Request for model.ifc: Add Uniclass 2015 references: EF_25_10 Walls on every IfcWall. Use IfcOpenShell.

First a look at what the model holds.

```python
import ifcopenshell

model = ifcopenshell.open("model.ifc")
print(model.schema)
print("classifications:", [c.Name for c in model.by_type("IfcClassification")])
for ifc_class in ("IfcDoor", "IfcRoof", "IfcStair", "IfcWall", "IfcWindow"):
    print(ifc_class, len(model.by_type(ifc_class)))
```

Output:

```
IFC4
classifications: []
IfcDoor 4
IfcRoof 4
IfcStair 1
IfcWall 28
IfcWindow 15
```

```python
import ifcopenshell
import ifcopenshell.api.classification

model = ifcopenshell.open("model.ifc")

system = ifcopenshell.api.classification.add_classification(model, classification="Uniclass 2015")

codes = {
    "IfcWall": ("EF_25_10", "Walls"),
}
for ifc_class, (code, name) in codes.items():
    products = model.by_type(ifc_class)
    ifcopenshell.api.classification.add_reference(
        model, products=products, classification=system, identification=code, name=name
    )
    print(code, len(products))

model.write("model_edited.ifc")
```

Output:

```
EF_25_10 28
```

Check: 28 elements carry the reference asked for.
